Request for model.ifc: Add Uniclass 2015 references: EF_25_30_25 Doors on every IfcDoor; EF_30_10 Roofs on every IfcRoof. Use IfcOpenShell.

First a look at what the model holds.

```python
import ifcopenshell

model = ifcopenshell.open("model.ifc")
print(model.schema)
print("classifications:", [c.Name for c in model.by_type("IfcClassification")])
for ifc_class in ("IfcDoor", "IfcRoof", "IfcStair", "IfcWall", "IfcWindow"):
    print(ifc_class, len(model.by_type(ifc_class)))
```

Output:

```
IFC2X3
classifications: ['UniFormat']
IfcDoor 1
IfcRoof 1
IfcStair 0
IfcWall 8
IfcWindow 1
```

```python
import ifcopenshell
import ifcopenshell.api.classification

model = ifcopenshell.open("model.ifc")

# IFC2X3 requires Source and Edition and has no link from the project to the system.
system = model.create_entity("IfcClassification", Source="NBS", Edition="2015", Name="Uniclass 2015")

codes = {
    "IfcDoor": ("EF_25_30_25", "Doors"),
    "IfcRoof": ("EF_30_10", "Roofs"),
}
for ifc_class, (code, name) in codes.items():
    products = model.by_type(ifc_class)
    ifcopenshell.api.classification.add_reference(
        model, products=products, classification=system, identification=code, name=name
    )
    print(code, len(products))

model.write("model_rev.ifc")
```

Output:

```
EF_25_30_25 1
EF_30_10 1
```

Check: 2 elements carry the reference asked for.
